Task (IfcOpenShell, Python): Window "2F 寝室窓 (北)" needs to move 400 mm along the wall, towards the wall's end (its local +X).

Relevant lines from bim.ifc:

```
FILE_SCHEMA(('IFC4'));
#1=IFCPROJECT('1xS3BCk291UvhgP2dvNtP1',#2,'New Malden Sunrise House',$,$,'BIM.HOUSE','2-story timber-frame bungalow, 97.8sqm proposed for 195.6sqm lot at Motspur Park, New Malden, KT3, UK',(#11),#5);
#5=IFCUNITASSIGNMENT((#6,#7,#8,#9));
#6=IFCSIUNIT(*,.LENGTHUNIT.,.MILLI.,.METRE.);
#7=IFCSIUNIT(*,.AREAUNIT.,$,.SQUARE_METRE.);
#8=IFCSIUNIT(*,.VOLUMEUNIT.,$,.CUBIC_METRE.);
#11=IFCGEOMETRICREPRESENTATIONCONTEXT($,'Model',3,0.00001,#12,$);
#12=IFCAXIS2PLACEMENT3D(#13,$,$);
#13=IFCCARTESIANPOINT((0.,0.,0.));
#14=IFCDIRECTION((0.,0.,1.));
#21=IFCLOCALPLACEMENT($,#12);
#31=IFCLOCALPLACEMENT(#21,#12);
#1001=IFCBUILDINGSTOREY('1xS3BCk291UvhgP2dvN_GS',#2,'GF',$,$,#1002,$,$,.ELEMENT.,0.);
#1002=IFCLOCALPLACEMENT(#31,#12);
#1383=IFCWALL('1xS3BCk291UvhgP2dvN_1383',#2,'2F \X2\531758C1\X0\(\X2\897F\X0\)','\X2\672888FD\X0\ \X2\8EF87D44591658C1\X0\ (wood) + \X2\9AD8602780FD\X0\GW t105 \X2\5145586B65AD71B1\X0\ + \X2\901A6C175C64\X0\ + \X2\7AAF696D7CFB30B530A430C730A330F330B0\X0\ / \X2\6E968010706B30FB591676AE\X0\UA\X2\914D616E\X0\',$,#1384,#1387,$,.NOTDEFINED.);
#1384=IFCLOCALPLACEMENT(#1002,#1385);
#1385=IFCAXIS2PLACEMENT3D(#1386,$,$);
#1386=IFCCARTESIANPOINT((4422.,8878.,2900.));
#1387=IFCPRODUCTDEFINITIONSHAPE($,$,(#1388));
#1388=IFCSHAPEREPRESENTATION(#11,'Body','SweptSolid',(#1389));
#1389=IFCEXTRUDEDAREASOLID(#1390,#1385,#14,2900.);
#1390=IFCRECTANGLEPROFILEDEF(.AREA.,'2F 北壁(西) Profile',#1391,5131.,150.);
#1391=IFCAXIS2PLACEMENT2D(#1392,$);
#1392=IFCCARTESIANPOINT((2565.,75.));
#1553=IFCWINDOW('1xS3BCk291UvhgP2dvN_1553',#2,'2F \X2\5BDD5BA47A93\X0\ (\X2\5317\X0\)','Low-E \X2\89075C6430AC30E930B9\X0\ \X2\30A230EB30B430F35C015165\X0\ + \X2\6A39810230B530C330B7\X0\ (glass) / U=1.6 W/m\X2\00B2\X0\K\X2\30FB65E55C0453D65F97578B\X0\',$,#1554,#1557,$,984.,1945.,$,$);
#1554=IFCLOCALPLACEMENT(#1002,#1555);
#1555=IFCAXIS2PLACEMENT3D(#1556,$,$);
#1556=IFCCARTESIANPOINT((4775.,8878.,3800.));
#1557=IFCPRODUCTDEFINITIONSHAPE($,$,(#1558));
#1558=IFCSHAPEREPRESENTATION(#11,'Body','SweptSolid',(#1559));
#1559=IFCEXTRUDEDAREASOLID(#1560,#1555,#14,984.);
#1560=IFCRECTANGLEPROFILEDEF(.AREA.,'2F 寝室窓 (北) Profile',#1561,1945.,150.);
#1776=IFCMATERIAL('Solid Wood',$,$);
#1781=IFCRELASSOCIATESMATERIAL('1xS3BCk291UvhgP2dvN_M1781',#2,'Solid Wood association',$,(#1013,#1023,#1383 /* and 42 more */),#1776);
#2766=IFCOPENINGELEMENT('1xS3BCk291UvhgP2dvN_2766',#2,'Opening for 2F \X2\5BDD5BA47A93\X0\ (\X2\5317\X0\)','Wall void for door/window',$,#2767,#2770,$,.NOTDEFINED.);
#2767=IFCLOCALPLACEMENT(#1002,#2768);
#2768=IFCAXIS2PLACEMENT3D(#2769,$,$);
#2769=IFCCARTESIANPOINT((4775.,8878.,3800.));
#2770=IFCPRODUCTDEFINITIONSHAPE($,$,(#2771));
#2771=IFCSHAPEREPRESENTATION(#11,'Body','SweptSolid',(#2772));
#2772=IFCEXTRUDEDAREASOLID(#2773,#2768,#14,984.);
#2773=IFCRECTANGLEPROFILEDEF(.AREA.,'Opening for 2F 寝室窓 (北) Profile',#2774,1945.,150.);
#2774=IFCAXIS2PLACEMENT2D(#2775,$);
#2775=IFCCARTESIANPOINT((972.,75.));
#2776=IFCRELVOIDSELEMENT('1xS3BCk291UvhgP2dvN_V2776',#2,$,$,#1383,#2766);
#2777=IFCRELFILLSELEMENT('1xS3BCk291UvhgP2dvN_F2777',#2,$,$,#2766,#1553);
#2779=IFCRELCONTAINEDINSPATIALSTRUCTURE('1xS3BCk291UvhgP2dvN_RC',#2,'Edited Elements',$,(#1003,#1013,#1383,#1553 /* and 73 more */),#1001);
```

```python
import ifcopenshell
import ifcopenshell.api.geometry
import ifcopenshell.util.placement
import ifcopenshell.util.unit

model = ifcopenshell.open("bim.ifc")
unit_scale = ifcopenshell.util.unit.calculate_unit_scale(model)

window = model.by_guid("1xS3BCk291UvhgP2dvN_1553")
opening = window.FillsVoids[0].RelatingOpeningElement
wall = opening.VoidsElements[0].RelatingBuildingElement

wall_matrix = ifcopenshell.util.placement.get_local_placement(wall.ObjectPlacement)
shift = wall_matrix[:3, 0] * 0.4 / unit_scale
before = ifcopenshell.util.placement.get_local_placement(window.ObjectPlacement)[:3, 3].copy()

# The window is not placed relative to its opening, so move both.
for product in (opening, window):
    matrix = ifcopenshell.util.placement.get_local_placement(product.ObjectPlacement)
    matrix[:3, 3] += shift
    ifcopenshell.api.geometry.edit_object_placement(model, product=product, matrix=matrix, is_si=False)

after = ifcopenshell.util.placement.get_local_placement(window.ObjectPlacement)[:3, 3]
print("window moved by", (after - before).round(3) + 0.0)

model.write("bim_v2.ifc")
```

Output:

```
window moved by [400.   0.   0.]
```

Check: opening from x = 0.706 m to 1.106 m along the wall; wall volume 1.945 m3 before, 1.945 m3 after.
